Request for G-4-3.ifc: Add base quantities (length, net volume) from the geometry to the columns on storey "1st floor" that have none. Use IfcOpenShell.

First a look at what the model holds.

```python
import ifcopenshell
import ifcopenshell.util.element
import ifcopenshell.util.unit

model = ifcopenshell.open("G-4-3.ifc")
print(model.schema)
for unit_type in ("LENGTHUNIT", "AREAUNIT", "VOLUMEUNIT"):
    print(unit_type, ifcopenshell.util.unit.calculate_unit_scale(model, unit_type))
storey = next(s for s in model.by_type("IfcBuildingStorey") if s.Name == "1st floor")
columns = [e for e in ifcopenshell.util.element.get_decomposition(storey) if e.is_a("IfcColumn")]
for e in sorted(columns, key=lambda e: e.id()):
    print(e.id(), e.is_a(), e.Name, list(ifcopenshell.util.element.get_psets(e, qtos_only=True)), sep=" | ")
```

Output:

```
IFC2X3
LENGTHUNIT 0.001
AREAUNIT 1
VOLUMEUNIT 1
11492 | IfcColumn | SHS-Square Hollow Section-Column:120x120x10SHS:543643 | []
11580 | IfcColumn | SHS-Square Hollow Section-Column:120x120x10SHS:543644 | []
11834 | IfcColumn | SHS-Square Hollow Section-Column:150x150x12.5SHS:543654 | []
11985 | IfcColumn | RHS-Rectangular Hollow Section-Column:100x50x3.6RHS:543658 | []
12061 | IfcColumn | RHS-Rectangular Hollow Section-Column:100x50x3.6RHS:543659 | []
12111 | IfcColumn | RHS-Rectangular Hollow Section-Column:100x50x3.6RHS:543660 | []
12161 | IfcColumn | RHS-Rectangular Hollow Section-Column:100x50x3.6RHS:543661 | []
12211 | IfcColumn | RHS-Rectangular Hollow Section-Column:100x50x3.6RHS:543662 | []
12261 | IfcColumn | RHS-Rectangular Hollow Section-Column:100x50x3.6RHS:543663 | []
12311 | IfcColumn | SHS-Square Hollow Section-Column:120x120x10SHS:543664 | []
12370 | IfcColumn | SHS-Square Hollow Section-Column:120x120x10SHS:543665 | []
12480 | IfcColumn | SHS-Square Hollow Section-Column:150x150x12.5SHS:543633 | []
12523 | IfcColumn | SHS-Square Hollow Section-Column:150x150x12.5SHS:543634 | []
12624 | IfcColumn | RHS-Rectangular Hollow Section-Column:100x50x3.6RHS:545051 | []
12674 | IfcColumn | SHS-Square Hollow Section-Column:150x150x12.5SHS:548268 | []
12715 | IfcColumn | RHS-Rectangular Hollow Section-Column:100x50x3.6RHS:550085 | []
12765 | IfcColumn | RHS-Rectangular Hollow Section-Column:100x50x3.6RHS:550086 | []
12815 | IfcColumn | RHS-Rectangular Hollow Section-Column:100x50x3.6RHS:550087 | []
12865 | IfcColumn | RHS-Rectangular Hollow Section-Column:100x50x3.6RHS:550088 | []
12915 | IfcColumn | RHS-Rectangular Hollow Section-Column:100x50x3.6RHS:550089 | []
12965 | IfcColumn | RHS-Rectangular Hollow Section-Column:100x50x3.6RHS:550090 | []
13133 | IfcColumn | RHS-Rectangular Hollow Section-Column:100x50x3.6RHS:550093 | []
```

```python
import ifcopenshell
import ifcopenshell.api.pset
import ifcopenshell.geom
import ifcopenshell.util.element
import ifcopenshell.util.shape
import ifcopenshell.util.unit

model = ifcopenshell.open("G-4-3.ifc")
unit_scale = ifcopenshell.util.unit.calculate_unit_scale(model)
volume_scale = ifcopenshell.util.unit.calculate_unit_scale(model, "VOLUMEUNIT")
settings = ifcopenshell.geom.settings()

storey = next(s for s in model.by_type("IfcBuildingStorey") if s.Name == "1st floor")
columns = [e for e in ifcopenshell.util.element.get_decomposition(storey) if e.is_a("IfcColumn")]

for e in sorted(columns, key=lambda e: e.id()):
    if ifcopenshell.util.element.get_psets(e, qtos_only=True, should_inherit=False):
        continue
    # Geometry comes back in metres, in the element's own axes.
    shape = ifcopenshell.geom.create_shape(settings, e)
    values = {
        "Length": ifcopenshell.util.shape.get_z(shape.geometry) / unit_scale,
        "NetVolume": ifcopenshell.util.shape.get_volume(shape.geometry) / volume_scale,
    }
    qto = ifcopenshell.api.pset.add_qto(model, product=e, name="BaseQuantities")
    ifcopenshell.api.pset.edit_qto(model, qto=qto, properties=values)
    print(e.id(), {k: round(v, 3) for k, v in values.items()})

model.write("G-4-3-out.ifc")
```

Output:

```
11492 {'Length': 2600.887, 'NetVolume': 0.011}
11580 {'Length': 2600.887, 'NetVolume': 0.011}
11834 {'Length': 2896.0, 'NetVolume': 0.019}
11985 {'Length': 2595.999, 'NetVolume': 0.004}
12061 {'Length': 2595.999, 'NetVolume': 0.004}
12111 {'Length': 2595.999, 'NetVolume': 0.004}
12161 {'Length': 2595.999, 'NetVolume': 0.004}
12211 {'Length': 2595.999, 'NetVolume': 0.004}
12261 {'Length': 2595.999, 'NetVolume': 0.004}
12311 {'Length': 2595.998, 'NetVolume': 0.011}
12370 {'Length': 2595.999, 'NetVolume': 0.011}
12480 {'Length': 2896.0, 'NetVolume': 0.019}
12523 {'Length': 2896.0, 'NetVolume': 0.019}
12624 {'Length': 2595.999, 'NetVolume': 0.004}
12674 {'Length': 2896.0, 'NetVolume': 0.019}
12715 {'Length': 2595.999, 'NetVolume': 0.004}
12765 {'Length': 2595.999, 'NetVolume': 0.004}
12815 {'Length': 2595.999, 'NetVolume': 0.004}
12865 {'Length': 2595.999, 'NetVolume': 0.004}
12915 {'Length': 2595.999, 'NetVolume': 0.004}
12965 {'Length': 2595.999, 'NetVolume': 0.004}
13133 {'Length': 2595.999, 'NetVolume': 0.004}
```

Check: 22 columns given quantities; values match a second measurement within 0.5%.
